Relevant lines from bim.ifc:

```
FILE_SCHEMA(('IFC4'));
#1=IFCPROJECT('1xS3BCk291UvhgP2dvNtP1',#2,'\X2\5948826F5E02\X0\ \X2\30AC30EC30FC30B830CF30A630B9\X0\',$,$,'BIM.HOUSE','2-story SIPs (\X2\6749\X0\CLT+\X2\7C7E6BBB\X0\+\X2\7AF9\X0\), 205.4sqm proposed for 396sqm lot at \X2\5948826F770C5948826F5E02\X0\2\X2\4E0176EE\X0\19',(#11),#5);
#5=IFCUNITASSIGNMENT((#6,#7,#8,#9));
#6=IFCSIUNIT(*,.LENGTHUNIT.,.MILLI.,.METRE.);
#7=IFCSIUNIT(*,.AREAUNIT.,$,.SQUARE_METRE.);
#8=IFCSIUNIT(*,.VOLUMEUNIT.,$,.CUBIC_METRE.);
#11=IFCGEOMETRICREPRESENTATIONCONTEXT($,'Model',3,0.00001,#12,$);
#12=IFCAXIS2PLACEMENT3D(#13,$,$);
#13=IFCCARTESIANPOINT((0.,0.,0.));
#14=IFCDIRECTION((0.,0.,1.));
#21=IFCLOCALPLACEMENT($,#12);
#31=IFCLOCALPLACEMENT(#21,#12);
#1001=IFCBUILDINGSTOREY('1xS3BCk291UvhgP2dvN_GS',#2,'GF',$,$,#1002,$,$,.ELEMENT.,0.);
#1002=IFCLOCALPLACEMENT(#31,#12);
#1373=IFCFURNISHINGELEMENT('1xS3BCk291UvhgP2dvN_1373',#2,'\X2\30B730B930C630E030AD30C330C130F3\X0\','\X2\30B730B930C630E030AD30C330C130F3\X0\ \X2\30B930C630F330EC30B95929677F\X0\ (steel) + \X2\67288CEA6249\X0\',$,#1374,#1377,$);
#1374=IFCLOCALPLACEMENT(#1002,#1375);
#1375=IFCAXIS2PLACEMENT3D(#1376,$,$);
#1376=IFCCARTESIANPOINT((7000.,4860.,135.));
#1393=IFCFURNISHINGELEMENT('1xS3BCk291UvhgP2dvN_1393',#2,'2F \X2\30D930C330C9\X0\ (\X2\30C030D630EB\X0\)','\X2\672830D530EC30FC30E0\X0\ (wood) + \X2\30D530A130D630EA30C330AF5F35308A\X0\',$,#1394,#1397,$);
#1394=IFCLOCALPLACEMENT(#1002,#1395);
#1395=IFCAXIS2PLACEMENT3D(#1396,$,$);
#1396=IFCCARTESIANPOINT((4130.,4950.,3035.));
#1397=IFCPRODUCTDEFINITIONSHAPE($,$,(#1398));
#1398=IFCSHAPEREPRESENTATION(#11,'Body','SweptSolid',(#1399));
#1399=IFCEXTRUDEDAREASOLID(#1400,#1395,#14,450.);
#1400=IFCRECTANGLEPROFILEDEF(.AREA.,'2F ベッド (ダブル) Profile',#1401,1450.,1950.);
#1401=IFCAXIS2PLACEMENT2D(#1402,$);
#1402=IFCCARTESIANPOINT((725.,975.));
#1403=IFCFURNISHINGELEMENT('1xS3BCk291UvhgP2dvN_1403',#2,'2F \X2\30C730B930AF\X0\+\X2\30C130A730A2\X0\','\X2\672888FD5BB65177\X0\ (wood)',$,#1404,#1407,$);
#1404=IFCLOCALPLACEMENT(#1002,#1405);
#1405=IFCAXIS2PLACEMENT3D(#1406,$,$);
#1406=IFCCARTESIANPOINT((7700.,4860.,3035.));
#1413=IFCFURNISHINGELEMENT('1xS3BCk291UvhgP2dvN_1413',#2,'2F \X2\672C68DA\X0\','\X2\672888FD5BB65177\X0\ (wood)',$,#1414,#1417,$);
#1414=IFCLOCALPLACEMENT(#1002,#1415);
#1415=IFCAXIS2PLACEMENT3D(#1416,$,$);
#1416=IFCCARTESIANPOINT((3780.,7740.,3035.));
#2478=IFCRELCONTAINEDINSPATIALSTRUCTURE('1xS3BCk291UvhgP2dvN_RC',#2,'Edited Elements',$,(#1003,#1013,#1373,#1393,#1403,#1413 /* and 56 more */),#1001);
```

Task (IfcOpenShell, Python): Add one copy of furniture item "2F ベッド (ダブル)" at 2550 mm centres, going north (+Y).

```python
import numpy as np
import ifcopenshell
import ifcopenshell.api.geometry
import ifcopenshell.api.root
import ifcopenshell.util.element
import ifcopenshell.util.placement

model = ifcopenshell.open("bim.ifc")


def reuse_history(source, copy):
    """copy_class also copies each property set's owner history, people and application; keep the originals."""
    for rel in copy.IsDefinedBy:
        if rel.is_a("IfcRelDefinesByProperties") and (history := rel.RelatingPropertyDefinition.OwnerHistory):
            rel.RelatingPropertyDefinition.OwnerHistory = source.OwnerHistory
            ifcopenshell.util.element.remove_deep2(model, history)


source = model.by_guid("1xS3BCk291UvhgP2dvN_1393")
base = ifcopenshell.util.placement.get_local_placement(source.ObjectPlacement)
step = np.array([0.0, 1.0, 0.0]) * 2550.0

for i in range(1, 2):
    copy = ifcopenshell.api.root.copy_class(model, product=source)
    copy.Representation = ifcopenshell.util.element.copy_deep(
        model, source.Representation, exclude=["IfcGeometricRepresentationContext", "IfcRepresentationMap"]
    )
    reuse_history(source, copy)
    matrix = base.copy()
    matrix[:3, 3] += i * step
    print("added at", matrix[:3, 3].round(3) + 0.0)
    ifcopenshell.api.geometry.edit_object_placement(model, product=copy, matrix=matrix, is_si=False)

model.write("bim_edited.ifc")
```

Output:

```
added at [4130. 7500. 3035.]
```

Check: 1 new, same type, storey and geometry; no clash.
